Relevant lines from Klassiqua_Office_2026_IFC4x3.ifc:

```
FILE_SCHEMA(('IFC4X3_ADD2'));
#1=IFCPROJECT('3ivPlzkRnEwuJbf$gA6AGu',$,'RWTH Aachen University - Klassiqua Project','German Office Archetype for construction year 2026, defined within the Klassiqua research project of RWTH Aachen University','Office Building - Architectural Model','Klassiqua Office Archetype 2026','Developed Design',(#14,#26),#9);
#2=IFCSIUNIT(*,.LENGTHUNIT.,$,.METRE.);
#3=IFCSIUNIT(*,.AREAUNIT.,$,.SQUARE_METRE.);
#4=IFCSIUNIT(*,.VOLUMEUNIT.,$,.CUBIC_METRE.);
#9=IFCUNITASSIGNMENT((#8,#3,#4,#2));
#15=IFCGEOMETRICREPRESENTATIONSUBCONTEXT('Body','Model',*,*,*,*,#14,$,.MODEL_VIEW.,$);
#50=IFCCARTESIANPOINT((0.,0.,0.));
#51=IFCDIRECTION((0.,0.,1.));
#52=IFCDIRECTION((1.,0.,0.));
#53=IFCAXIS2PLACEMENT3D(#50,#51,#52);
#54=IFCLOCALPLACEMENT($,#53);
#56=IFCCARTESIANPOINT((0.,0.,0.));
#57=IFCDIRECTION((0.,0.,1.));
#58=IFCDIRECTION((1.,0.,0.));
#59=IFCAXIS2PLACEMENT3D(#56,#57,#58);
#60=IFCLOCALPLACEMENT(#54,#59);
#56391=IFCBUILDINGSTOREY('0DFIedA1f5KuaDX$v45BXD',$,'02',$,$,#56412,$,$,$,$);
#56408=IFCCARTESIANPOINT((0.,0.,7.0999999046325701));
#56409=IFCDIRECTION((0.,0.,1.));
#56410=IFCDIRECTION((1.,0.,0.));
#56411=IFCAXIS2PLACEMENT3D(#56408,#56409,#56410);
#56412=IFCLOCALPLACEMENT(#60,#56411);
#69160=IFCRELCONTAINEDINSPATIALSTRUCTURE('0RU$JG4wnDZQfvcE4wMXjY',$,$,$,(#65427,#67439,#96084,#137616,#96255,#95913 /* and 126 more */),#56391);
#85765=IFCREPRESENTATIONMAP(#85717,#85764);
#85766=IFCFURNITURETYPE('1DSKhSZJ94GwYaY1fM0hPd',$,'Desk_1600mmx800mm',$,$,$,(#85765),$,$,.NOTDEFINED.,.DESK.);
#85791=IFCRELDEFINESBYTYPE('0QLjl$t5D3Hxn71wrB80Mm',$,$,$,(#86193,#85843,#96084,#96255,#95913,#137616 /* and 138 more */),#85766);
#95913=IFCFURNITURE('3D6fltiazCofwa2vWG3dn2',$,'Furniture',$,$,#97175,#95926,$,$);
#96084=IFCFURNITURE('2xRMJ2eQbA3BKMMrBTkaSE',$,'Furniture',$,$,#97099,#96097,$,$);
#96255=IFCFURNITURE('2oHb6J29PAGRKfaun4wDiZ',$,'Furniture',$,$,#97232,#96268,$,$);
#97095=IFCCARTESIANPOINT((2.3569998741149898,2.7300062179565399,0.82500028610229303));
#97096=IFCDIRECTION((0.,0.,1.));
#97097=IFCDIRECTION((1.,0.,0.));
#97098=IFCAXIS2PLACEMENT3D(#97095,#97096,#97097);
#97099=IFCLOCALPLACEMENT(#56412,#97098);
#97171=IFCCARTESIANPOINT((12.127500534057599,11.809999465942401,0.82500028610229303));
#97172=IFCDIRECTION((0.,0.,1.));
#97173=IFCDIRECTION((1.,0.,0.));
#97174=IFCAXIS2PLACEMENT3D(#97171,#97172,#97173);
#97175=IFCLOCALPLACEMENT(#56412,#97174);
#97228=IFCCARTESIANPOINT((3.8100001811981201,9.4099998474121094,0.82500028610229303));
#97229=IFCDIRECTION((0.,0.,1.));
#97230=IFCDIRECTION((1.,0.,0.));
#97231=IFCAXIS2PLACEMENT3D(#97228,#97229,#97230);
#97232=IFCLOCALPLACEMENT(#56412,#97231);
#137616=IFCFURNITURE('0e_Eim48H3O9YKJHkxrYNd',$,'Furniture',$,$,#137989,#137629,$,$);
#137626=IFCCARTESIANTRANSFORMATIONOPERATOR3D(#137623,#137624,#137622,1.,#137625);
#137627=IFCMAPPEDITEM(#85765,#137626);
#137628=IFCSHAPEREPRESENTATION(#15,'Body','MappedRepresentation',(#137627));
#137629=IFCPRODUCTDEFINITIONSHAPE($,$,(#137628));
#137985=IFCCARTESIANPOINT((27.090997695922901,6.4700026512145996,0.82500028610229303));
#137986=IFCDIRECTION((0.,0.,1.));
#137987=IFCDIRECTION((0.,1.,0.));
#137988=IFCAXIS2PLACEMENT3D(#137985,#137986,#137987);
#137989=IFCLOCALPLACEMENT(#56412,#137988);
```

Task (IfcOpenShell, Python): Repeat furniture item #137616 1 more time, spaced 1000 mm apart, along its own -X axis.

```python
import ifcopenshell
import ifcopenshell.api.geometry
import ifcopenshell.api.root
import ifcopenshell.util.element
import ifcopenshell.util.placement
import ifcopenshell.util.unit

model = ifcopenshell.open("Klassiqua_Office_2026_IFC4x3.ifc")
unit_scale = ifcopenshell.util.unit.calculate_unit_scale(model)

source = model.by_guid("0e_Eim48H3O9YKJHkxrYNd")
base = ifcopenshell.util.placement.get_local_placement(source.ObjectPlacement)
step = -base[:3, 0] * 1 / unit_scale

for i in range(1, 2):
    copy = ifcopenshell.api.root.copy_class(model, product=source)
    copy.Representation = ifcopenshell.util.element.copy_deep(
        model, source.Representation, exclude=["IfcGeometricRepresentationContext", "IfcRepresentationMap"]
    )
    matrix = base.copy()
    matrix[:3, 3] += i * step
    print("added at", matrix[:3, 3].round(3) + 0.0)
    ifcopenshell.api.geometry.edit_object_placement(model, product=copy, matrix=matrix, is_si=False)

model.write("Klassiqua_Office_2026_IFC4x3_v2.ifc")
```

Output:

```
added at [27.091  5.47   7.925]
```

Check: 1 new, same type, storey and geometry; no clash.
